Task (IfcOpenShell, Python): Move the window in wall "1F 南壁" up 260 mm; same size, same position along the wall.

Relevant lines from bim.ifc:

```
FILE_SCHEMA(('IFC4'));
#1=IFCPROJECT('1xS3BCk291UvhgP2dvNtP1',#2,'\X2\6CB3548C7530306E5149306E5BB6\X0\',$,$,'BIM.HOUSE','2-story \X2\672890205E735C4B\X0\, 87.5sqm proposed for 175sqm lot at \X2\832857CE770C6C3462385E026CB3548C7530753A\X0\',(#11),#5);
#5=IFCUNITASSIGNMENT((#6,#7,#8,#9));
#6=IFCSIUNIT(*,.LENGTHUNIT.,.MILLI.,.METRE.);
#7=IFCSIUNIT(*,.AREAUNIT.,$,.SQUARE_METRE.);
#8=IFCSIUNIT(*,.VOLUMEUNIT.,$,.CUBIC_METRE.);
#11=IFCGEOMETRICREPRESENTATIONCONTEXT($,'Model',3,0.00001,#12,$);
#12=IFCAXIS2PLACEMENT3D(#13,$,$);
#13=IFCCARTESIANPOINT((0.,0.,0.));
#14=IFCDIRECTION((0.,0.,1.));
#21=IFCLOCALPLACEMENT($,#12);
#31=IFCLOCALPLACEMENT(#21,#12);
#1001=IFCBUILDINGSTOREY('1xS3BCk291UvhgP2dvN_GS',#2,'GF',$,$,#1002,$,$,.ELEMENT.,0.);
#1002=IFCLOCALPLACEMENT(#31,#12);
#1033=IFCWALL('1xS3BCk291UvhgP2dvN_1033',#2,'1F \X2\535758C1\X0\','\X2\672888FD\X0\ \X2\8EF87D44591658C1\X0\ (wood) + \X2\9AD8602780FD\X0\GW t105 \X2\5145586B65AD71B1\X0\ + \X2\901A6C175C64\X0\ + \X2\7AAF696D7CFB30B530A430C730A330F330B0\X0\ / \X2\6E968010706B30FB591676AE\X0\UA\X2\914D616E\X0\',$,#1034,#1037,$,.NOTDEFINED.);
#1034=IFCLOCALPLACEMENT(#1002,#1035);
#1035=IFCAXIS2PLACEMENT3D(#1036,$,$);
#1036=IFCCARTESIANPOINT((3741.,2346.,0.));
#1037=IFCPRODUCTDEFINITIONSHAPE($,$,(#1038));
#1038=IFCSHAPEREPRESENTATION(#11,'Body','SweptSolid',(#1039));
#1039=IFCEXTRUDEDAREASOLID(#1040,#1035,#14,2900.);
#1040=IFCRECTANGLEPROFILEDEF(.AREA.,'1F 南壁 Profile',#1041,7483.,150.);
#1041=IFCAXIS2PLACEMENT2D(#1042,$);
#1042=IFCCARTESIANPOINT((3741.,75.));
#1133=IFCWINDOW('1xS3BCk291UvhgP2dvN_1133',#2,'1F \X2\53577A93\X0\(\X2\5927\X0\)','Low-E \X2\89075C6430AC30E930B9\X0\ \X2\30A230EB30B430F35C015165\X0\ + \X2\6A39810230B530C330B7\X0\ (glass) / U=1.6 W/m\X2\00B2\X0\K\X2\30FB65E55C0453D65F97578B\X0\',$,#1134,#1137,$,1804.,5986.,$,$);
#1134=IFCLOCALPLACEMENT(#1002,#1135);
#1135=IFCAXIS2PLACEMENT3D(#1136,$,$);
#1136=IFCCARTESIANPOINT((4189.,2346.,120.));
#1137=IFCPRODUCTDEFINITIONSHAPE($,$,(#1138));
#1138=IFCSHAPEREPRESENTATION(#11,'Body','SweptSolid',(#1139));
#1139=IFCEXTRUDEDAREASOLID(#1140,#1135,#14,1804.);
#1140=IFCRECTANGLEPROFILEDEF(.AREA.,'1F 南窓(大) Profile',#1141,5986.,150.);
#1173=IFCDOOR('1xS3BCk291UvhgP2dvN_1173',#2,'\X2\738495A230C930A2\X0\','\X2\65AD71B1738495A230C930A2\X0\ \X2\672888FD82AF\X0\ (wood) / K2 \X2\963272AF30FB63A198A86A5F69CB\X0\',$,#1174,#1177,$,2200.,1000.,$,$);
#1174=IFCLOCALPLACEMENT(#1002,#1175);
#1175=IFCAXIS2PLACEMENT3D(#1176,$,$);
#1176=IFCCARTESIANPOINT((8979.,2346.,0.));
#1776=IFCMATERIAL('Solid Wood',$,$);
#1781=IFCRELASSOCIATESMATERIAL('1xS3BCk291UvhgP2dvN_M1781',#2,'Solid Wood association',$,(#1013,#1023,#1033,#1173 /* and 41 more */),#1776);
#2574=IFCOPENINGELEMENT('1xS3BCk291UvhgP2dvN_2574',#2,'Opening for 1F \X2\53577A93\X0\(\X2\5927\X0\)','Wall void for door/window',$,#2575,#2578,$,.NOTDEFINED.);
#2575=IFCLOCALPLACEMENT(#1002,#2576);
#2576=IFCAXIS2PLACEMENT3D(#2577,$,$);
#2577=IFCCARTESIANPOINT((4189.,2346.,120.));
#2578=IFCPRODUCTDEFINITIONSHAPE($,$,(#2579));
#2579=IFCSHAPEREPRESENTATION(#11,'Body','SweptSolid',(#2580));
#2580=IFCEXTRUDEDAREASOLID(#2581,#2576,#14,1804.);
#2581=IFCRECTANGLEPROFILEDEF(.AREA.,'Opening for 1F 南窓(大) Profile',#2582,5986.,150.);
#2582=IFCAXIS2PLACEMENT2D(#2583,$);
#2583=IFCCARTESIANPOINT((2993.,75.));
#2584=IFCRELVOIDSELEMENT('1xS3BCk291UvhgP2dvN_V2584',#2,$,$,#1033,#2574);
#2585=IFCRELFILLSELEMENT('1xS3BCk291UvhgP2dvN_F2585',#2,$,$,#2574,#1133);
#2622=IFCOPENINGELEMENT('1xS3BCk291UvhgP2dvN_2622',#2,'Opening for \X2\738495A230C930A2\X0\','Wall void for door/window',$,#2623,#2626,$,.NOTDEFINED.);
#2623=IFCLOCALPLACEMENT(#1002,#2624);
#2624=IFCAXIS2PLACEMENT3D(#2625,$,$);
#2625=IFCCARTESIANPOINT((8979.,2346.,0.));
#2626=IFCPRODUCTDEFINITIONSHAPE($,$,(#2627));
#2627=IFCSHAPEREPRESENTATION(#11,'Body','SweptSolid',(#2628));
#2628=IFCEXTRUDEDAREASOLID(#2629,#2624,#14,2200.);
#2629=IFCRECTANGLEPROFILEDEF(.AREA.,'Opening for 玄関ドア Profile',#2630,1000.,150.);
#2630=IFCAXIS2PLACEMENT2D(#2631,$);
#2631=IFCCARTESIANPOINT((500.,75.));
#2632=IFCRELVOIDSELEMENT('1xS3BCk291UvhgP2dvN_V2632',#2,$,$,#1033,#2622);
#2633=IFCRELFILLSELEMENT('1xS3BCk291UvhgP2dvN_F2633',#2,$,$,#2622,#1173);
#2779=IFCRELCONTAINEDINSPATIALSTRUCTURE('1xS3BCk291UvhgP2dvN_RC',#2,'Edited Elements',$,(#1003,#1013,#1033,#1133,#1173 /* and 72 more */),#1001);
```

```python
import numpy as np
import ifcopenshell
import ifcopenshell.api.geometry
import ifcopenshell.util.placement
import ifcopenshell.util.unit

model = ifcopenshell.open("bim.ifc")
unit_scale = ifcopenshell.util.unit.calculate_unit_scale(model)

window = model.by_guid("1xS3BCk291UvhgP2dvN_1133")
opening = window.FillsVoids[0].RelatingOpeningElement
dz = 0.26 / unit_scale

shift = np.array([0.0, 0.0, dz])
# The window is not placed relative to its opening, so move both.
for product in (opening, window):
    matrix = ifcopenshell.util.placement.get_local_placement(product.ObjectPlacement)
    matrix[:3, 3] += shift
    ifcopenshell.api.geometry.edit_object_placement(model, product=product, matrix=matrix, is_si=False)

print(f"moved by {dz * unit_scale:+.3f} m")

model.write("bim_v2.ifc")
```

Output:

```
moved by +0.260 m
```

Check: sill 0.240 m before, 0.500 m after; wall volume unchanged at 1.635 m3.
